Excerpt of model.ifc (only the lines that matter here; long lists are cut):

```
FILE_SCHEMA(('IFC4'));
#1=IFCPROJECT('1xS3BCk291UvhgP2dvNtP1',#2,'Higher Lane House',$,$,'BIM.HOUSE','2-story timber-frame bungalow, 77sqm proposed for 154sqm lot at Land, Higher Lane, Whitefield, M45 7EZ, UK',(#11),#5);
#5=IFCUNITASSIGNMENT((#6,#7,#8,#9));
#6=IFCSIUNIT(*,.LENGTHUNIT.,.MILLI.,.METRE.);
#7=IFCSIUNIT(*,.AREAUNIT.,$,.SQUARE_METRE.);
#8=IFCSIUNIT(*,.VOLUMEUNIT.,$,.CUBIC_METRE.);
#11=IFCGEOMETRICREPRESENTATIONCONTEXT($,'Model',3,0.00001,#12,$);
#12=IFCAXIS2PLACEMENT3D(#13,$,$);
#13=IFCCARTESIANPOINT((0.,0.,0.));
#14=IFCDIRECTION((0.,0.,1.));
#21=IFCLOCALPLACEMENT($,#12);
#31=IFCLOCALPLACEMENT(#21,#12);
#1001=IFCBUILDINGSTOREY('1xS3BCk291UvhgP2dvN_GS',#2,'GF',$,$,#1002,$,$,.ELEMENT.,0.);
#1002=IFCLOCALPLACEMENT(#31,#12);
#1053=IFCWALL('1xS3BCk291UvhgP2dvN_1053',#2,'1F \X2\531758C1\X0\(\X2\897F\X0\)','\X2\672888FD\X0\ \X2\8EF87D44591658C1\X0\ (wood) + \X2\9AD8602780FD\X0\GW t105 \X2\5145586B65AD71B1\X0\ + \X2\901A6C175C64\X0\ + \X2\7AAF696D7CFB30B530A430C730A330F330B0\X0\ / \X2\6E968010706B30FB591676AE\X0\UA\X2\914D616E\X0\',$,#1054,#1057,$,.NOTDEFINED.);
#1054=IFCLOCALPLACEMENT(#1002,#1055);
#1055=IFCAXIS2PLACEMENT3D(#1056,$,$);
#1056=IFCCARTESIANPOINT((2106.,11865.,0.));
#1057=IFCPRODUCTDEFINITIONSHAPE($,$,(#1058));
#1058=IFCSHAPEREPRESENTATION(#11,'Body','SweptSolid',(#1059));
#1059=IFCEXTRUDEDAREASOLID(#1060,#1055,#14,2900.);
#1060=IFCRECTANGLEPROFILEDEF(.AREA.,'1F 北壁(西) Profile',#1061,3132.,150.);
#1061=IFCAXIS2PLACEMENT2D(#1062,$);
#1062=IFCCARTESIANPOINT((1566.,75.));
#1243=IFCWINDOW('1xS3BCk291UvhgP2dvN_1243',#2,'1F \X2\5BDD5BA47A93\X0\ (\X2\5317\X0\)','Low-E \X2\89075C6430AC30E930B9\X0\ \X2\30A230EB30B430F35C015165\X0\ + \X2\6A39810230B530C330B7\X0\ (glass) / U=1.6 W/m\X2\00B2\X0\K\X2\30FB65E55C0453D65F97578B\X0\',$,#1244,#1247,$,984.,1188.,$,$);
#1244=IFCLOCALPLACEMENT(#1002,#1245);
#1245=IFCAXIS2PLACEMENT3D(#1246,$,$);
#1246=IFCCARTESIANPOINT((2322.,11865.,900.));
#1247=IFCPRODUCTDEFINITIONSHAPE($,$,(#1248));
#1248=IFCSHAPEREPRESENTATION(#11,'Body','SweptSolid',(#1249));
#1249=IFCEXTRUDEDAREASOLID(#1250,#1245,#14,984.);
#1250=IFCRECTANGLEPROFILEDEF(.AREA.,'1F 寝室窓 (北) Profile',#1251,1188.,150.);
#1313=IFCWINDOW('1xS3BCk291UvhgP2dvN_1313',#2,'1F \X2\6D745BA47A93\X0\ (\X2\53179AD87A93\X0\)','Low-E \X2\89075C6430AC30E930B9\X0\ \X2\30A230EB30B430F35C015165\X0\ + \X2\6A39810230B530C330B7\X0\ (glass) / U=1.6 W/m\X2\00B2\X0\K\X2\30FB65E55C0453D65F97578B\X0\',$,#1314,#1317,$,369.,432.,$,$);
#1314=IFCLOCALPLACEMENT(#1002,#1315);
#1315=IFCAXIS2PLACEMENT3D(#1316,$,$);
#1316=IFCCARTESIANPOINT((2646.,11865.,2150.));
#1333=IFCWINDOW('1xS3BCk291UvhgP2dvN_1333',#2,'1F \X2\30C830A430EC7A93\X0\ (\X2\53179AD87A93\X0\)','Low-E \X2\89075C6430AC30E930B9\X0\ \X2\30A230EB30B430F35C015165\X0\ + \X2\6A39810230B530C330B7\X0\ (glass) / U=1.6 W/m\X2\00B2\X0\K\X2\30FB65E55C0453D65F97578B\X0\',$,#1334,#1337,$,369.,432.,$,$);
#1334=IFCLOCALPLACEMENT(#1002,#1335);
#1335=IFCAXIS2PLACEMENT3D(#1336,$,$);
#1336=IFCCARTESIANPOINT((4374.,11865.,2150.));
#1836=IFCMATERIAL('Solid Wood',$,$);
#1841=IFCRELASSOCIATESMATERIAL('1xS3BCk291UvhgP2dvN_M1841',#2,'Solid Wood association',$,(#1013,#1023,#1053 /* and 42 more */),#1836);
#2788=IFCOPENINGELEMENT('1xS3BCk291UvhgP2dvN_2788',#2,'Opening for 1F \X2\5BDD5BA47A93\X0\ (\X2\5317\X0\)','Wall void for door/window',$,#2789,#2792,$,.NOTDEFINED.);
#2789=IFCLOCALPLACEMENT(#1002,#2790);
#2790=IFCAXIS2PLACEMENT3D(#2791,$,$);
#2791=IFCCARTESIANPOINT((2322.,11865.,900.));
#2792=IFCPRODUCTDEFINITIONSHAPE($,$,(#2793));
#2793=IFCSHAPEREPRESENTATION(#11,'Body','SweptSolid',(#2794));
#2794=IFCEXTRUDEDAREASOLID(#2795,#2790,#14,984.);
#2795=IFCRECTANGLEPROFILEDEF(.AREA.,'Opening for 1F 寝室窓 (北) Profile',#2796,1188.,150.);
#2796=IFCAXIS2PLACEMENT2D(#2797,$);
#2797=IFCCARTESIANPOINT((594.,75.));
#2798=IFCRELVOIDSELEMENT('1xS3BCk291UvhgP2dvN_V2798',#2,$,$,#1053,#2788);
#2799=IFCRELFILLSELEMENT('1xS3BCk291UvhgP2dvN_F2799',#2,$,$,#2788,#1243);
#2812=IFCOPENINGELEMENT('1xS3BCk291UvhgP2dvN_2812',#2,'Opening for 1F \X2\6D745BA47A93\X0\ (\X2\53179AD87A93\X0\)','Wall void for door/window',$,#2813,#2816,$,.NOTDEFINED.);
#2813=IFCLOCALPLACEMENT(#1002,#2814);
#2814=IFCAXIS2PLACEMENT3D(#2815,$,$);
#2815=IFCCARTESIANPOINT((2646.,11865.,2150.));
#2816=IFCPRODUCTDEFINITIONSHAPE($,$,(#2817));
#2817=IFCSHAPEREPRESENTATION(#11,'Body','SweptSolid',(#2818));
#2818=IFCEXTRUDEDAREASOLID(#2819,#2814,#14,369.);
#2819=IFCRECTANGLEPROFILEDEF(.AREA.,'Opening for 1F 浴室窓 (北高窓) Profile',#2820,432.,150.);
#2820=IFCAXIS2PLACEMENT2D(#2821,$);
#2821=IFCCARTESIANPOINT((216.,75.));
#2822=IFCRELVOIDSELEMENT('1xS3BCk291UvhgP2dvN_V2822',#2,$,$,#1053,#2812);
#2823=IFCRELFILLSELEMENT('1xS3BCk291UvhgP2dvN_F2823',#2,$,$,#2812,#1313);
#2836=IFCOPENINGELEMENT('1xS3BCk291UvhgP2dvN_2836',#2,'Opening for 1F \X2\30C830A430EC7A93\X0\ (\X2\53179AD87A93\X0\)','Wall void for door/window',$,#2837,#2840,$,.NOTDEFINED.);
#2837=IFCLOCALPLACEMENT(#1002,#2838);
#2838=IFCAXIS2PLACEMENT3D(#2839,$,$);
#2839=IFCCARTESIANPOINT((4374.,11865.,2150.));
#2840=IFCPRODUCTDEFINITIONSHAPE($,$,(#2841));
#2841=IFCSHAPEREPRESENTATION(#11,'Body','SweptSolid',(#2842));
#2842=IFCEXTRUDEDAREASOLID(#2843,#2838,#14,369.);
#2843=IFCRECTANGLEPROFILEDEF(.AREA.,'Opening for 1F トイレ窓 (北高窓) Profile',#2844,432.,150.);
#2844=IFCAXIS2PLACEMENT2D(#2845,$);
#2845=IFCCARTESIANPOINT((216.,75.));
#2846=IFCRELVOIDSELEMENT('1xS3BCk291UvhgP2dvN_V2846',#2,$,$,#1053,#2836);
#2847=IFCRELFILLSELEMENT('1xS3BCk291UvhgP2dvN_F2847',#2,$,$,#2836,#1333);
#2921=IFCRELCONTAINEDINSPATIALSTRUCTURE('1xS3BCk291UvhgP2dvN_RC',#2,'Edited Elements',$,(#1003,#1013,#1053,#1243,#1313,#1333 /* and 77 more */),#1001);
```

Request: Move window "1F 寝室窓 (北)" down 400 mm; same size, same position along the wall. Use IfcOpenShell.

```python
import numpy as np
import ifcopenshell
import ifcopenshell.api.geometry
import ifcopenshell.util.placement
import ifcopenshell.util.unit

model = ifcopenshell.open("model.ifc")
unit_scale = ifcopenshell.util.unit.calculate_unit_scale(model)

window = model.by_guid("1xS3BCk291UvhgP2dvN_1243")
opening = window.FillsVoids[0].RelatingOpeningElement
dz = -400.0

shift = np.array([0.0, 0.0, dz])
# The window is not placed relative to its opening, so move both.
for product in (opening, window):
    matrix = ifcopenshell.util.placement.get_local_placement(product.ObjectPlacement)
    matrix[:3, 3] += shift
    ifcopenshell.api.geometry.edit_object_placement(model, product=product, matrix=matrix, is_si=False)

print(f"moved by {dz * unit_scale:+.3f} m")

model.write("model-out.ifc")
```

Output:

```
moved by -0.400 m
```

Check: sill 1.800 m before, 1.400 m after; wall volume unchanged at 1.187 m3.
